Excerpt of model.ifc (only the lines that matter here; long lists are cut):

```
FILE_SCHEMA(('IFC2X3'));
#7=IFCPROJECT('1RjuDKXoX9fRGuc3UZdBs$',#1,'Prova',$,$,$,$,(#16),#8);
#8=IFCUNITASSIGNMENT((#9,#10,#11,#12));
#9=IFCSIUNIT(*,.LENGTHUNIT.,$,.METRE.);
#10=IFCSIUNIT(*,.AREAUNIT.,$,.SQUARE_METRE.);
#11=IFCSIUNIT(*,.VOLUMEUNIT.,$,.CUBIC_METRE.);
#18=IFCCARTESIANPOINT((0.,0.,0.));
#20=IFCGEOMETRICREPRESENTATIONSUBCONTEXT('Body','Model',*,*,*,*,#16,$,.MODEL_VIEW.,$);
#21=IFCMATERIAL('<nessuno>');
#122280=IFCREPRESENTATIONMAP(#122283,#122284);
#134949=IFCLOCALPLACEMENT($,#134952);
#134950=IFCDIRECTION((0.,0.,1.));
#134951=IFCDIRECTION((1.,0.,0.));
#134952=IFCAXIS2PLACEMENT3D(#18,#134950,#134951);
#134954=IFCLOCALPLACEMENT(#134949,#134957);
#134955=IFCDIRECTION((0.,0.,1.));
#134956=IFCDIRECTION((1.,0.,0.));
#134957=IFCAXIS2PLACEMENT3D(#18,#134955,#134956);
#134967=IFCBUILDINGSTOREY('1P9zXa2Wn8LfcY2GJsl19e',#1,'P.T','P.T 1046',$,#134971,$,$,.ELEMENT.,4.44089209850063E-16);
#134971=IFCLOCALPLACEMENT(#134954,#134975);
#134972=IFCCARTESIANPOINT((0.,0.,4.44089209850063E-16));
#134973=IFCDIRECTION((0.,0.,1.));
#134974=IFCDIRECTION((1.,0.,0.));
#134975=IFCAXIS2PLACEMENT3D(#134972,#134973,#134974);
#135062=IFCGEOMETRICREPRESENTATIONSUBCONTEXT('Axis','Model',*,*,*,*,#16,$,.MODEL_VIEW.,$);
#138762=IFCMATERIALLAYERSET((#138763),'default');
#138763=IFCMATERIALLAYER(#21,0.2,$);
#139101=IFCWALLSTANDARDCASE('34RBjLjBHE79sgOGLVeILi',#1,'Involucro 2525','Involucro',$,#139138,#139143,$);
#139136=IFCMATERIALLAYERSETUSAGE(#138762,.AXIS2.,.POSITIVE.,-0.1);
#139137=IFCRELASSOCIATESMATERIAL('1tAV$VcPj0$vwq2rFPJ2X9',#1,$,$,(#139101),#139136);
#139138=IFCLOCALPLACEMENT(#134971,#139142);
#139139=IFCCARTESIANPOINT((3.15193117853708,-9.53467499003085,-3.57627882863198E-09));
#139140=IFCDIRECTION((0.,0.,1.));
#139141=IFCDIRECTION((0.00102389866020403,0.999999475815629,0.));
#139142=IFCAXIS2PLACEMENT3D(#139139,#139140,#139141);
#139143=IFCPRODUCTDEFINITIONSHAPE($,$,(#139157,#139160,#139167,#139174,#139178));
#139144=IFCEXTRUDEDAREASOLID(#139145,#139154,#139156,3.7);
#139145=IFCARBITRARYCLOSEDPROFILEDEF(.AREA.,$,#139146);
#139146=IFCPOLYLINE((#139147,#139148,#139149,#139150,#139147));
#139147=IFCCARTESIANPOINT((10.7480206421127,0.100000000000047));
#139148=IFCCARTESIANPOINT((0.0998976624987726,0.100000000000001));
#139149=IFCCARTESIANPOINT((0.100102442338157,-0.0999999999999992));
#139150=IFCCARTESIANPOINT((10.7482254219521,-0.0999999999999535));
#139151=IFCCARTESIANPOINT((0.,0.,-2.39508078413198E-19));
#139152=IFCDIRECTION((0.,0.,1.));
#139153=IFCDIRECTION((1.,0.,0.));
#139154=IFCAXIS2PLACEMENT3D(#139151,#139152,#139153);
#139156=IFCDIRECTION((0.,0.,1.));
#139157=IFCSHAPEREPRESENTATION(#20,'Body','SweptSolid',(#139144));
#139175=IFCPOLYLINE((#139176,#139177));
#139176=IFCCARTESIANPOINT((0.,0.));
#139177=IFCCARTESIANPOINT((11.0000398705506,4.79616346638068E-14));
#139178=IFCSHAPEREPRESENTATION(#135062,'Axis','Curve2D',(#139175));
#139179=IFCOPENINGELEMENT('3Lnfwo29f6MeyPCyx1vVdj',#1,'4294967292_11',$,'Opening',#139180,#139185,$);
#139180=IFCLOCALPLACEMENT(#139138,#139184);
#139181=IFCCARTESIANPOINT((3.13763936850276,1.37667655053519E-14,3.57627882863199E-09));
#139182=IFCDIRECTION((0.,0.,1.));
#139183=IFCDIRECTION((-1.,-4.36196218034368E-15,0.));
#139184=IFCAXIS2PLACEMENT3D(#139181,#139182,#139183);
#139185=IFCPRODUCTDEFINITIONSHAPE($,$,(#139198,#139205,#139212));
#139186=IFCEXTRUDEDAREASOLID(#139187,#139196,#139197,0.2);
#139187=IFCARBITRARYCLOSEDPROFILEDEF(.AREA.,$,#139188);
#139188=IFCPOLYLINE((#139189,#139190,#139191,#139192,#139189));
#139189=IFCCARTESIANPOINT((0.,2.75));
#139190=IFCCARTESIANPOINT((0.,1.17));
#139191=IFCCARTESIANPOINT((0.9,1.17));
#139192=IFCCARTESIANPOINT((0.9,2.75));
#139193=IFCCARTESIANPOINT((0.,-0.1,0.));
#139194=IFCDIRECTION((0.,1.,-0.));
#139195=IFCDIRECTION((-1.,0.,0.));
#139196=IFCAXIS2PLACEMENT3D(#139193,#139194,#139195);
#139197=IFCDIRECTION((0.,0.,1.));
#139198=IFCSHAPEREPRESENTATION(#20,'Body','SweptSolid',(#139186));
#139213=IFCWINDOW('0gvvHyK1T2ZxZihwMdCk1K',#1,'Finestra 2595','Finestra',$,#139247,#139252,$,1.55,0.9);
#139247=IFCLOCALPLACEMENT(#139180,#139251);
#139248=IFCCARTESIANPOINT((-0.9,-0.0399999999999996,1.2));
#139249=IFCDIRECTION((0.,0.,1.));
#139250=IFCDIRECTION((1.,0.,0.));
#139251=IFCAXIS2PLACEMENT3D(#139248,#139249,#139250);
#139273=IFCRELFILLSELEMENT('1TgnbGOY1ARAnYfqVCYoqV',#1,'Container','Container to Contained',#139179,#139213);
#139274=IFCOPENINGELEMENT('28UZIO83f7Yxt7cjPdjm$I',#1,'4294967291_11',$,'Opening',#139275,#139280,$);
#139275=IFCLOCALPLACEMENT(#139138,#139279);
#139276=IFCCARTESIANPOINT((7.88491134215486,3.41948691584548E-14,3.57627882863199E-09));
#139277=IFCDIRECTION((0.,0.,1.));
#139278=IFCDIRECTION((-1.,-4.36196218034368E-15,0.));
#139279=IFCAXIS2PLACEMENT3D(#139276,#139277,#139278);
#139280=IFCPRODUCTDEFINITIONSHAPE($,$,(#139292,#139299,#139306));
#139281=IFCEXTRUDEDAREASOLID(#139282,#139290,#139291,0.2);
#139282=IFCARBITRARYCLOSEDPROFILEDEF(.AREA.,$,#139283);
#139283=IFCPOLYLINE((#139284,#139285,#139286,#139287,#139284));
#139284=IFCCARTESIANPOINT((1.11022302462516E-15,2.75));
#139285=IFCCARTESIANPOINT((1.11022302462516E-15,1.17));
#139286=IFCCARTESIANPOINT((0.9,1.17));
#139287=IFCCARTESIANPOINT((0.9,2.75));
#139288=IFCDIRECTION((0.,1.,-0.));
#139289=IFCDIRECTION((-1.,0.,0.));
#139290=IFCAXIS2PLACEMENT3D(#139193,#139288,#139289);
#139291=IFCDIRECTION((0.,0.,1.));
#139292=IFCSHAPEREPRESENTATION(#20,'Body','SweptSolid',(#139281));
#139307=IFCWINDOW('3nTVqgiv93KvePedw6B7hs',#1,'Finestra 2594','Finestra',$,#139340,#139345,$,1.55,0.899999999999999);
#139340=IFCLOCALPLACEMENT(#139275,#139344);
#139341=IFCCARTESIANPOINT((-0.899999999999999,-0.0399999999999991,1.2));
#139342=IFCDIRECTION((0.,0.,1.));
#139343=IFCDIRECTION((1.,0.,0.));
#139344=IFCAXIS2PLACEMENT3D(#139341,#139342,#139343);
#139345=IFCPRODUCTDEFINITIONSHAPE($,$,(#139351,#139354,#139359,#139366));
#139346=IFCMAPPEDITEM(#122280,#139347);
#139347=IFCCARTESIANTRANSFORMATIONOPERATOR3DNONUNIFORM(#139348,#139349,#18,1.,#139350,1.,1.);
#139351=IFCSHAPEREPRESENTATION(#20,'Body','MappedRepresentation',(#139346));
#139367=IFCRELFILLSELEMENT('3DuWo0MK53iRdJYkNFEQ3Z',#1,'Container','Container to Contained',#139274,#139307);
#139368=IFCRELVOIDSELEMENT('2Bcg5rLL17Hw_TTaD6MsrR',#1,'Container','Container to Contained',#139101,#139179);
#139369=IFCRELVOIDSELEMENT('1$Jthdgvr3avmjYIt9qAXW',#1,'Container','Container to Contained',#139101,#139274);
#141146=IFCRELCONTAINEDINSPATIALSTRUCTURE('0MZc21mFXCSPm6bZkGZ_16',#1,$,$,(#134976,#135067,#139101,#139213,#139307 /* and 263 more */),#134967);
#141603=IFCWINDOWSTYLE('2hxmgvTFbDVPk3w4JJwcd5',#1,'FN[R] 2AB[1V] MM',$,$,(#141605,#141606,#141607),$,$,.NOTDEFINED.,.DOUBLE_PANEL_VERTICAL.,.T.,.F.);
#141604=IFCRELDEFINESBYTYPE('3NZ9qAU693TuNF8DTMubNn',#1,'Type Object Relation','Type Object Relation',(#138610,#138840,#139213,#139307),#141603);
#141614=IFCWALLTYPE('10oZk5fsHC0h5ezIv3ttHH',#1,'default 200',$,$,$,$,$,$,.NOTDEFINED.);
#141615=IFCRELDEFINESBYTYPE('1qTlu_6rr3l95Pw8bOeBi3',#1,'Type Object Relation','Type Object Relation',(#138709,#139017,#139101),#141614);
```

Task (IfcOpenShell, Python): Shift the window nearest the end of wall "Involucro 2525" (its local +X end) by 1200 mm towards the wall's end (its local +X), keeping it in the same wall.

```python
import ifcopenshell
import ifcopenshell.api.geometry
import ifcopenshell.util.placement
import ifcopenshell.util.unit

model = ifcopenshell.open("model.ifc")
unit_scale = ifcopenshell.util.unit.calculate_unit_scale(model)

window = model.by_guid("3nTVqgiv93KvePedw6B7hs")
opening = window.FillsVoids[0].RelatingOpeningElement
wall = opening.VoidsElements[0].RelatingBuildingElement

wall_matrix = ifcopenshell.util.placement.get_local_placement(wall.ObjectPlacement)
shift = wall_matrix[:3, 0] * 1.2 / unit_scale
before = ifcopenshell.util.placement.get_local_placement(window.ObjectPlacement)[:3, 3].copy()

# The window is placed relative to its opening, so it follows when the opening moves.
matrix = ifcopenshell.util.placement.get_local_placement(opening.ObjectPlacement)
matrix[:3, 3] += shift
ifcopenshell.api.geometry.edit_object_placement(
    model, product=opening, matrix=matrix, is_si=False, should_transform_children=True
)

after = ifcopenshell.util.placement.get_local_placement(window.ObjectPlacement)[:3, 3]
print("window moved by", (after - before).round(3) + 0.0)

model.write("model_v2.ifc")
```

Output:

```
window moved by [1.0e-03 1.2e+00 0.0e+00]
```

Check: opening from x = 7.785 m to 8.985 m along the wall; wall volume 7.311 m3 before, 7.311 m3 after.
